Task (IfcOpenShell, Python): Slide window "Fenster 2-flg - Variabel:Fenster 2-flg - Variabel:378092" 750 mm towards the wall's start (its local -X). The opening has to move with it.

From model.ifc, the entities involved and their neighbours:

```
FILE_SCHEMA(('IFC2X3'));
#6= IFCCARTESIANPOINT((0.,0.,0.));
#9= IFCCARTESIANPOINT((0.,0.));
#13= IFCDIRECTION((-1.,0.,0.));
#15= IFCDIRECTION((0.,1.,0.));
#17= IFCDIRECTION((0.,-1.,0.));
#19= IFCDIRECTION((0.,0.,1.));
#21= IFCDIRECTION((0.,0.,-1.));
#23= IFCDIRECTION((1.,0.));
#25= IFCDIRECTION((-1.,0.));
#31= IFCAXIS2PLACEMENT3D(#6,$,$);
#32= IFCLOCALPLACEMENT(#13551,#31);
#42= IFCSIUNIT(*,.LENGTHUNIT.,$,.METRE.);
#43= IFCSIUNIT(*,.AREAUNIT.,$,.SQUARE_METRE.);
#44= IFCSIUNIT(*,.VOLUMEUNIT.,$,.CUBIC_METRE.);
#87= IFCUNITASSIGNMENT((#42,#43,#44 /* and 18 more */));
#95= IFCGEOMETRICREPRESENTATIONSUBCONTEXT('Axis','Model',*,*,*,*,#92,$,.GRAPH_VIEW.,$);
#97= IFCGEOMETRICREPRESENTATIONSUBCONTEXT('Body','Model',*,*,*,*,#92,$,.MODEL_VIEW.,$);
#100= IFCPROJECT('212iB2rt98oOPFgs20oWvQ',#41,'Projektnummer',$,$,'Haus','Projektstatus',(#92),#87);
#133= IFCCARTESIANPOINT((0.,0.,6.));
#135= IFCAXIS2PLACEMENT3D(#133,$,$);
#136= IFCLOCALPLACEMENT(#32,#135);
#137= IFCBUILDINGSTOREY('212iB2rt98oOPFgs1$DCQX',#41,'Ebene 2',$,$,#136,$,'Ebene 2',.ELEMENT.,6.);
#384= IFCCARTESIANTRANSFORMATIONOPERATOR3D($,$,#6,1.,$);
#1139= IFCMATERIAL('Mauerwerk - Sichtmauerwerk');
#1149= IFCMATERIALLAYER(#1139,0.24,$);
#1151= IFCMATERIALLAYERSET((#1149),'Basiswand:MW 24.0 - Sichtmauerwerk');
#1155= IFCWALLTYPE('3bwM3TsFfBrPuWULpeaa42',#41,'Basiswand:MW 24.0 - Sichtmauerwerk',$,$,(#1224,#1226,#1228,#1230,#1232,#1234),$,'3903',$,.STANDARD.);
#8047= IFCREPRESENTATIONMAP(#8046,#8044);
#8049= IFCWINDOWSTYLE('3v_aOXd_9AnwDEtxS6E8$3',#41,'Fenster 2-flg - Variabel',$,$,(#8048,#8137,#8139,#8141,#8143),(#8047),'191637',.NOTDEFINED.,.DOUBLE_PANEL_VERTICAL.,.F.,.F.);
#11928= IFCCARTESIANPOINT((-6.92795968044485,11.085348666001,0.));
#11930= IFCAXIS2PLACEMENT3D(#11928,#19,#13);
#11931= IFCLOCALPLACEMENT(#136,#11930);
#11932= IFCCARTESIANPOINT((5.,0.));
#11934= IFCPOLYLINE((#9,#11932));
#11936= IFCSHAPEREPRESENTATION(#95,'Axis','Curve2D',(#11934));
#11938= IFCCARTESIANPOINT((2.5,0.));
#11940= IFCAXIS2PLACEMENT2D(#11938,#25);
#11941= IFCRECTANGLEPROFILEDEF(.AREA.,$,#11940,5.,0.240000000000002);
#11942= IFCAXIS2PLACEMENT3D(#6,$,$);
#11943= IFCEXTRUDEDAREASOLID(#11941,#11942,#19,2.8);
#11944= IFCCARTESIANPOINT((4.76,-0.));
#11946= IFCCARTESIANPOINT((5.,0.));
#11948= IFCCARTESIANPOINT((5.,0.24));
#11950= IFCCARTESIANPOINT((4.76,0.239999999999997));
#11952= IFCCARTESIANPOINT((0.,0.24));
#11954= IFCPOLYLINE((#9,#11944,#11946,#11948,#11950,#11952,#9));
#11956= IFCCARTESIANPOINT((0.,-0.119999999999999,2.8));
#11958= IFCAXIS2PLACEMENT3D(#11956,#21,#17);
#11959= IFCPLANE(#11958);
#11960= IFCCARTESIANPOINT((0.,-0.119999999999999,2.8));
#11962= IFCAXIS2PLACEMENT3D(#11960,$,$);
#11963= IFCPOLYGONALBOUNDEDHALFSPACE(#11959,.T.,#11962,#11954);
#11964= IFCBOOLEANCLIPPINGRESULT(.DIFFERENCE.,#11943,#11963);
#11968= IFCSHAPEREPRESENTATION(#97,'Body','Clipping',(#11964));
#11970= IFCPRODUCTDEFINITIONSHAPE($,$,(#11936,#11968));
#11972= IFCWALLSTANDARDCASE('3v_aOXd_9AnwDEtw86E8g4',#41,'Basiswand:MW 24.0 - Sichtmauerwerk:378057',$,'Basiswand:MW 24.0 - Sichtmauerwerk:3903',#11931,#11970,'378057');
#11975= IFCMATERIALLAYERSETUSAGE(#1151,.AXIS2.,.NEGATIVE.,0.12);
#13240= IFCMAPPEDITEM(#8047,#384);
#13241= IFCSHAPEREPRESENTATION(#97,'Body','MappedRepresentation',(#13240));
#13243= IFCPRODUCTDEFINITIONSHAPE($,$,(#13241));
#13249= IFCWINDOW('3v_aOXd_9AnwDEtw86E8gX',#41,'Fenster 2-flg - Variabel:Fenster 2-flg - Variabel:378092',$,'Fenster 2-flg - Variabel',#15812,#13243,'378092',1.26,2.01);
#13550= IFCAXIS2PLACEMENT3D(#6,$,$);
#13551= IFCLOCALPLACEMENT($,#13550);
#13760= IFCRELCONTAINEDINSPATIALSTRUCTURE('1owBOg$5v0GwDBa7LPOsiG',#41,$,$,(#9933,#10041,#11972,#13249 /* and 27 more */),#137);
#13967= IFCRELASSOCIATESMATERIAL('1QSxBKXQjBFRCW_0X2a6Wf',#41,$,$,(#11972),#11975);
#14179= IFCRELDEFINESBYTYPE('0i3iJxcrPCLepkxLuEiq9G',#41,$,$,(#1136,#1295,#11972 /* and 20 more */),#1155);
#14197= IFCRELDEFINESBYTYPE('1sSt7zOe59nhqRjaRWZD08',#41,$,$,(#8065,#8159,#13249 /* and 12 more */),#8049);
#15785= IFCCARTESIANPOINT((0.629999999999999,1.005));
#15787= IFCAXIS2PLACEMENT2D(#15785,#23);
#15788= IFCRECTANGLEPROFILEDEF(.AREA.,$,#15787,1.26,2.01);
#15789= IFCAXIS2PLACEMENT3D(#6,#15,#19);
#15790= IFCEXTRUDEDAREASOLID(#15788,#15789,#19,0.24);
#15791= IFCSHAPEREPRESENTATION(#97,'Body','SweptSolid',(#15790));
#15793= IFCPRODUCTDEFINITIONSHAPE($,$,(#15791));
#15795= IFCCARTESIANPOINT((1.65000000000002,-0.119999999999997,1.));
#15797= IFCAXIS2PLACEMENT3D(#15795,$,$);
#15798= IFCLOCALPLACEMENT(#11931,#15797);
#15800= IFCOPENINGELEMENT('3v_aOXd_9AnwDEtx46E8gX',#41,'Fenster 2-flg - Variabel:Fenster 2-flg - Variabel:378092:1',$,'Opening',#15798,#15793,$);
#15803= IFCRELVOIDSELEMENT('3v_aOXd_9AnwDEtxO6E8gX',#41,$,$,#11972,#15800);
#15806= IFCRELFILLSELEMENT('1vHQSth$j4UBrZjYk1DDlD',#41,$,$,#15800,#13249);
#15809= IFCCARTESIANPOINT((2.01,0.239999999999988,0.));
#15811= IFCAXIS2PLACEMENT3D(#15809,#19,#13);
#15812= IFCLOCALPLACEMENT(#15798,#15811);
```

```python
import ifcopenshell
import ifcopenshell.api.geometry
import ifcopenshell.util.placement

model = ifcopenshell.open("model.ifc")

window = model.by_guid("3v_aOXd_9AnwDEtw86E8gX")
opening = window.FillsVoids[0].RelatingOpeningElement
wall = opening.VoidsElements[0].RelatingBuildingElement

wall_matrix = ifcopenshell.util.placement.get_local_placement(wall.ObjectPlacement)
shift = wall_matrix[:3, 0] * -0.75
before = ifcopenshell.util.placement.get_local_placement(window.ObjectPlacement)[:3, 3].copy()

# The window is placed relative to its opening, so it follows when the opening moves.
matrix = ifcopenshell.util.placement.get_local_placement(opening.ObjectPlacement)
matrix[:3, 3] += shift
ifcopenshell.api.geometry.edit_object_placement(
    model, product=opening, matrix=matrix, is_si=False, should_transform_children=True
)

after = ifcopenshell.util.placement.get_local_placement(window.ObjectPlacement)[:3, 3]
print("window moved by", (after - before).round(3) + 0.0)

model.write("model_updated.ifc")
```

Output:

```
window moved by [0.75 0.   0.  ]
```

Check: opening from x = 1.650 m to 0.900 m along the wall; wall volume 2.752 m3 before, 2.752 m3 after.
